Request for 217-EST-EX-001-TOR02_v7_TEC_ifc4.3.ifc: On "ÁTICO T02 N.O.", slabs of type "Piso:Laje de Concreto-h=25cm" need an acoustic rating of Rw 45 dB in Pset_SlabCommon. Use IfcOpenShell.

First a look at what the model holds.

```python
import ifcopenshell
import ifcopenshell.util.element

model = ifcopenshell.open("217-EST-EX-001-TOR02_v7_TEC_ifc4.3.ifc")
print(model.schema)
storey = next(s for s in model.by_type("IfcBuildingStorey") if s.Name == "ÁTICO T02 N.O.")
slabs = [e for e in ifcopenshell.util.element.get_decomposition(storey) if e.is_a("IfcSlab")]
seen = {}
for e in slabs:
    element_type = ifcopenshell.util.element.get_type(e)
    key = (element_type.Name if element_type != e and element_type else None, ifcopenshell.util.element.get_pset(e, "Pset_SlabCommon", "AcousticRating"))
    seen[key] = seen.get(key, 0) + 1
for (name, value), count in sorted(seen.items(), key=str):
    print(count, "x", name, "|", value)
```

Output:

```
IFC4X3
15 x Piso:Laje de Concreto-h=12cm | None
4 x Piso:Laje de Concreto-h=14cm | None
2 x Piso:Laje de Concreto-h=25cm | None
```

```python
import ifcopenshell
import ifcopenshell.api.pset
import ifcopenshell.util.element

model = ifcopenshell.open("217-EST-EX-001-TOR02_v7_TEC_ifc4.3.ifc")

storey = next(s for s in model.by_type("IfcBuildingStorey") if s.Name == "ÁTICO T02 N.O.")
slabs = [e for e in ifcopenshell.util.element.get_decomposition(storey) if e.is_a("IfcSlab")]

count = 0
for e in slabs:
    element_type = ifcopenshell.util.element.get_type(e)
    if element_type in (None, e) or element_type.Name != "Piso:Laje de Concreto-h=25cm":
        continue
    # add_pset returns the element's existing set when there is one.
    pset = ifcopenshell.api.pset.add_pset(model, product=e, name="Pset_SlabCommon")
    ifcopenshell.api.pset.edit_pset(model, pset=pset, properties={"AcousticRating": "Rw 45 dB"})
    count += 1

print(count, "slabs updated")

model.write("217-EST-EX-001-TOR02_v7_TEC_ifc4.3_rev.ifc")
```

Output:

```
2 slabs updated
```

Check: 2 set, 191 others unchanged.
